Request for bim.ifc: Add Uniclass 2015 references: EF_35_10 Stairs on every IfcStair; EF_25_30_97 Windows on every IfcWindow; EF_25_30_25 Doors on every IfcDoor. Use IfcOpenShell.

First a look at what the model holds.

```python
import ifcopenshell

model = ifcopenshell.open("bim.ifc")
print(model.schema)
print("classifications:", [c.Name for c in model.by_type("IfcClassification")])
for ifc_class in ("IfcDoor", "IfcRoof", "IfcStair", "IfcWall", "IfcWindow"):
    print(ifc_class, len(model.by_type(ifc_class)))
```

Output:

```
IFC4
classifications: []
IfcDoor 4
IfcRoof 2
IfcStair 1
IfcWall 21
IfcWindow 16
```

```python
import ifcopenshell
import ifcopenshell.api.classification

model = ifcopenshell.open("bim.ifc")

system = ifcopenshell.api.classification.add_classification(model, classification="Uniclass 2015")

codes = {
    "IfcStair": ("EF_35_10", "Stairs"),
    "IfcWindow": ("EF_25_30_97", "Windows"),
    "IfcDoor": ("EF_25_30_25", "Doors"),
}
for ifc_class, (code, name) in codes.items():
    products = model.by_type(ifc_class)
    ifcopenshell.api.classification.add_reference(
        model, products=products, classification=system, identification=code, name=name
    )
    print(code, len(products))

model.write("bim_edited.ifc")
```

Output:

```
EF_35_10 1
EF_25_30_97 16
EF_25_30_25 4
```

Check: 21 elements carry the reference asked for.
